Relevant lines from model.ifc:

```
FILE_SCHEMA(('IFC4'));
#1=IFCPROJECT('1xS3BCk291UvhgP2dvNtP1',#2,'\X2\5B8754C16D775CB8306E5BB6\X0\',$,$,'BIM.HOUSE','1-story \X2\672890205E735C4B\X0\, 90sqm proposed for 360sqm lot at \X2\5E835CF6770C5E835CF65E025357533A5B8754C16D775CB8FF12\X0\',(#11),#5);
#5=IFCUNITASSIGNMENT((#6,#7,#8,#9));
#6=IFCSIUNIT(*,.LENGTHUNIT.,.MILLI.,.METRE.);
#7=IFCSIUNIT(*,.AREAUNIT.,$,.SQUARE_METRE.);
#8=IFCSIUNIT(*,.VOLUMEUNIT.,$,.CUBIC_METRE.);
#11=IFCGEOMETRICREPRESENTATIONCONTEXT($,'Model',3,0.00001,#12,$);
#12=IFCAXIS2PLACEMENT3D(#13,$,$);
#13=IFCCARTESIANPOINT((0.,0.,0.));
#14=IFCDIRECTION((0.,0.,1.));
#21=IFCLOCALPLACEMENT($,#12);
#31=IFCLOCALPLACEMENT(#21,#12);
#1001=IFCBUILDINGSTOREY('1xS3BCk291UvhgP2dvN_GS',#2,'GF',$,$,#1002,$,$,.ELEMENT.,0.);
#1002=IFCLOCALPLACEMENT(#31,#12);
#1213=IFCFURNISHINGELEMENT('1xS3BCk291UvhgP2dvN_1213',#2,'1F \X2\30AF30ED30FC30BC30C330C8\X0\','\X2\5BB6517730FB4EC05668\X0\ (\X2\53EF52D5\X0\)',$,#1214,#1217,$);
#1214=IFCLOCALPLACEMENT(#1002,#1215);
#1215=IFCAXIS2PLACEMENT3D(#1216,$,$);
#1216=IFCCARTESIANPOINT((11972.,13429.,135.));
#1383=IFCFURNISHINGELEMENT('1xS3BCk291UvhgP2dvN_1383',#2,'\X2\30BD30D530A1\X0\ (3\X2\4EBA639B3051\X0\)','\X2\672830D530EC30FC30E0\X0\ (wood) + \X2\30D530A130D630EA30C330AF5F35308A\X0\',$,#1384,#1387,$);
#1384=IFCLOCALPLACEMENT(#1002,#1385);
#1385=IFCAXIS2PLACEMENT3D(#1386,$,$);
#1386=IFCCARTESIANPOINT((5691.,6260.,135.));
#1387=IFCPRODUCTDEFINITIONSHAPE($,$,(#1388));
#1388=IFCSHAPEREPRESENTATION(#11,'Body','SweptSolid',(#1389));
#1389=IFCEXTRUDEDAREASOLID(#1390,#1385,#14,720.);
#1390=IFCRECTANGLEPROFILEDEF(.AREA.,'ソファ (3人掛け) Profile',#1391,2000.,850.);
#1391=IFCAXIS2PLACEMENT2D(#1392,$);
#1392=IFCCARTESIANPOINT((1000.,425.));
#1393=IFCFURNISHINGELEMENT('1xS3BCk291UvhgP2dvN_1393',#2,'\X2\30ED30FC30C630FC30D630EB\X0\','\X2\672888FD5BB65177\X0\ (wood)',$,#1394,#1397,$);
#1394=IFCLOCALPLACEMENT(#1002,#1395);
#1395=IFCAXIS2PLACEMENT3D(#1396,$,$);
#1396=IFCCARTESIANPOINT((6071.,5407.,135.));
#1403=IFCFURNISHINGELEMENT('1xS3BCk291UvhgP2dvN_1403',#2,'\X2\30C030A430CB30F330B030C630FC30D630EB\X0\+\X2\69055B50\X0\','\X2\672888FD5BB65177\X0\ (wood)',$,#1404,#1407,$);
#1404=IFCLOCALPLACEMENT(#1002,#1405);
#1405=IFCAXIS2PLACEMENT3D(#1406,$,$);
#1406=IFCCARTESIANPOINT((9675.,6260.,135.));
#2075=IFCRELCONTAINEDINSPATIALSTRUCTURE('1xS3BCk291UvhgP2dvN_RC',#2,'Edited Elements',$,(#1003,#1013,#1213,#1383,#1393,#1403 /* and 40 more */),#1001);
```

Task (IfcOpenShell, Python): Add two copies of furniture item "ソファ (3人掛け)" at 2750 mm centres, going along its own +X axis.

```python
import ifcopenshell
import ifcopenshell.api.geometry
import ifcopenshell.api.root
import ifcopenshell.util.element
import ifcopenshell.util.placement

model = ifcopenshell.open("model.ifc")


def reuse_history(source, copy):
    """copy_class also copies each property set's owner history, people and application; keep the originals."""
    for rel in copy.IsDefinedBy:
        if rel.is_a("IfcRelDefinesByProperties") and (history := rel.RelatingPropertyDefinition.OwnerHistory):
            rel.RelatingPropertyDefinition.OwnerHistory = source.OwnerHistory
            ifcopenshell.util.element.remove_deep2(model, history)


source = model.by_guid("1xS3BCk291UvhgP2dvN_1383")
base = ifcopenshell.util.placement.get_local_placement(source.ObjectPlacement)
step = base[:3, 0] * 2750.0

for i in range(1, 3):
    copy = ifcopenshell.api.root.copy_class(model, product=source)
    copy.Representation = ifcopenshell.util.element.copy_deep(
        model, source.Representation, exclude=["IfcGeometricRepresentationContext", "IfcRepresentationMap"]
    )
    reuse_history(source, copy)
    matrix = base.copy()
    matrix[:3, 3] += i * step
    print("added at", matrix[:3, 3].round(3) + 0.0)
    ifcopenshell.api.geometry.edit_object_placement(model, product=copy, matrix=matrix, is_si=False)

model.write("model-out.ifc")
```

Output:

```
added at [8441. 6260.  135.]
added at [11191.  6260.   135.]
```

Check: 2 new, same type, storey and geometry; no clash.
